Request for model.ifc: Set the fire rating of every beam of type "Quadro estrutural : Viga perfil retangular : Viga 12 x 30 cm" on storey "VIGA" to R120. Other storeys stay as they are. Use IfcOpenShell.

First a look at what the model holds.

```python
import ifcopenshell
import ifcopenshell.util.element

model = ifcopenshell.open("model.ifc")
print(model.schema)
storey = next(s for s in model.by_type("IfcBuildingStorey") if s.Name == "VIGA")
beams = [e for e in ifcopenshell.util.element.get_decomposition(storey) if e.is_a("IfcBeam")]
seen = {}
for e in beams:
    element_type = ifcopenshell.util.element.get_type(e)
    key = (element_type.Name if element_type != e and element_type else None, ifcopenshell.util.element.get_pset(e, "Pset_BeamCommon", "FireRating"))
    seen[key] = seen.get(key, 0) + 1
for (name, value), count in sorted(seen.items(), key=str):
    print(count, "x", name, "|", value)
```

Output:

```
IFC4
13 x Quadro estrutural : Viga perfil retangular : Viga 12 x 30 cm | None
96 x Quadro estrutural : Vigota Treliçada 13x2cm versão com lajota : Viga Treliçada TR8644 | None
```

```python
import ifcopenshell
import ifcopenshell.api.pset
import ifcopenshell.util.element

model = ifcopenshell.open("model.ifc")

storey = next(s for s in model.by_type("IfcBuildingStorey") if s.Name == "VIGA")
beams = [e for e in ifcopenshell.util.element.get_decomposition(storey) if e.is_a("IfcBeam")]

count = 0
for e in beams:
    element_type = ifcopenshell.util.element.get_type(e)
    if element_type in (None, e) or element_type.Name != "Quadro estrutural : Viga perfil retangular : Viga 12 x 30 cm":
        continue
    # add_pset returns the element's existing set when there is one.
    pset = ifcopenshell.api.pset.add_pset(model, product=e, name="Pset_BeamCommon")
    ifcopenshell.api.pset.edit_pset(model, pset=pset, properties={"FireRating": "R120"})
    count += 1

print(count, "beams updated")

model.write("model-out.ifc")
```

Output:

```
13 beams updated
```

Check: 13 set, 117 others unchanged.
